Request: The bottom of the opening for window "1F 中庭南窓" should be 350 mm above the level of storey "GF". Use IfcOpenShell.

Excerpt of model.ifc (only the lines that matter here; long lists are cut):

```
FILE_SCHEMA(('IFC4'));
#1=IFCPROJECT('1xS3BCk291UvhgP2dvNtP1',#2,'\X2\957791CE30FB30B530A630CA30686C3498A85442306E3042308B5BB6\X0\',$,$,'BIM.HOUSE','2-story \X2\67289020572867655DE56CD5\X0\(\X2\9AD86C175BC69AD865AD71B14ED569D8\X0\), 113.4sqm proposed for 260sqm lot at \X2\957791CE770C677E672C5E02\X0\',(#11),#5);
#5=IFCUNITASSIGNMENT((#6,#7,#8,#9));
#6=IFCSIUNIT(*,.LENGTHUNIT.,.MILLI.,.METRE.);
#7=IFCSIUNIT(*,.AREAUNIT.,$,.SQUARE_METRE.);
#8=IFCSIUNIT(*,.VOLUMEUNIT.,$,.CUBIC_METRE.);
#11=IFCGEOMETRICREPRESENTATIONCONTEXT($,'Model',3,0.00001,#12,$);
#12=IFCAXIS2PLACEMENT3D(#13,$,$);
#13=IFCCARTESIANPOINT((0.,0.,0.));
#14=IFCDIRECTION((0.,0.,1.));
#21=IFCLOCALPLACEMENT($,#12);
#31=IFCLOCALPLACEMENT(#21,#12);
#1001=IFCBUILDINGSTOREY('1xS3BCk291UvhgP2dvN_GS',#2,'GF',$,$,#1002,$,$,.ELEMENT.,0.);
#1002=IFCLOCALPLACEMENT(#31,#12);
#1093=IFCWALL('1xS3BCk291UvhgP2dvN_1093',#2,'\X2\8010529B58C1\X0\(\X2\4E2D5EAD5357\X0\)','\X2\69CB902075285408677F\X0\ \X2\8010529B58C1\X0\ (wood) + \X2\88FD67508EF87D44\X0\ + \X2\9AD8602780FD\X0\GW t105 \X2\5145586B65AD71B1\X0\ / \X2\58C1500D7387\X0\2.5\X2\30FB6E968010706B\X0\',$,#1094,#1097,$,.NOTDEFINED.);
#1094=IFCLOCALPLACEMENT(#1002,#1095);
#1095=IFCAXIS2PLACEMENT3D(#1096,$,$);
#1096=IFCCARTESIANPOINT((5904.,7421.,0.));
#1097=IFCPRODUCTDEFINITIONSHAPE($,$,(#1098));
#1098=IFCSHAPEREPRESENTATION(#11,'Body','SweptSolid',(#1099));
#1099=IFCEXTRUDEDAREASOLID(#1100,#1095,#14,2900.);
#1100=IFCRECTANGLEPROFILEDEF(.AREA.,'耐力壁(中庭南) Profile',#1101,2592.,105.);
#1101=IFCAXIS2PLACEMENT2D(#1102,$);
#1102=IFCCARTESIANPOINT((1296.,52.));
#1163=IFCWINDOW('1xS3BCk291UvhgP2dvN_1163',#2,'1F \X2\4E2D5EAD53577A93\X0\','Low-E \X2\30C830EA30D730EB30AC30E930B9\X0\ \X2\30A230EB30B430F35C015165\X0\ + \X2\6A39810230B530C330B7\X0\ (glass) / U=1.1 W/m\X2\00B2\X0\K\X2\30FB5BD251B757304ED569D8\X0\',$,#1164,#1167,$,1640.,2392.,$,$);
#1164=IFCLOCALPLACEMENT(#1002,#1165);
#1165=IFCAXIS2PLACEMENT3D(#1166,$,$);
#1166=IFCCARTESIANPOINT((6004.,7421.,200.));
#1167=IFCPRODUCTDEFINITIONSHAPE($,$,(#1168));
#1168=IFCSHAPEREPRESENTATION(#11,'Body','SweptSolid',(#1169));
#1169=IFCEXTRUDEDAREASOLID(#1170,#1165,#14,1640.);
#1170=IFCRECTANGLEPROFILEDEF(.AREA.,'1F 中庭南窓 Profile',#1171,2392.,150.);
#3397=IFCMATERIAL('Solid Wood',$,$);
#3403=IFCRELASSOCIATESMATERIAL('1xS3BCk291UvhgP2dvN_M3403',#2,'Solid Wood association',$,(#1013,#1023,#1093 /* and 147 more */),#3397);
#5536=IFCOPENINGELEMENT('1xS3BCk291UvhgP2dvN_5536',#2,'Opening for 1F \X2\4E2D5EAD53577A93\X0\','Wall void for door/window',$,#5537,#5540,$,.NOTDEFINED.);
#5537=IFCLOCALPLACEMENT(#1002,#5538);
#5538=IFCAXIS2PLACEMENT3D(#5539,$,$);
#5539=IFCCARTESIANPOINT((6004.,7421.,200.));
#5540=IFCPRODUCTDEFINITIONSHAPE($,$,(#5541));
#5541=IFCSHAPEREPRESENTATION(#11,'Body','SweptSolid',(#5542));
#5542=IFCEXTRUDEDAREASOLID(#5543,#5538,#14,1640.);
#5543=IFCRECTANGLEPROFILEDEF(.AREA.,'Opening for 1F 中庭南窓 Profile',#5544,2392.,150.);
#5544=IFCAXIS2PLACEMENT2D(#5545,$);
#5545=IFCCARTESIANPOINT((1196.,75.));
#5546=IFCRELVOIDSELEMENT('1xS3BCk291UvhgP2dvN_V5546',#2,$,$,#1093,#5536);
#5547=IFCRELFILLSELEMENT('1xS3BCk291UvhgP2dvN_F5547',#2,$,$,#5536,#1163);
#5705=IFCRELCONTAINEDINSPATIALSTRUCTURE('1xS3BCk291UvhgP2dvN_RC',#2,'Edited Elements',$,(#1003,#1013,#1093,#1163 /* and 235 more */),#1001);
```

```python
import numpy as np
import ifcopenshell
import ifcopenshell.api.geometry
import ifcopenshell.geom
import ifcopenshell.util.element
import ifcopenshell.util.placement
import ifcopenshell.util.shape
import ifcopenshell.util.unit

model = ifcopenshell.open("model.ifc")
unit_scale = ifcopenshell.util.unit.calculate_unit_scale(model)

window = model.by_id(1163)
opening = window.FillsVoids[0].RelatingOpeningElement
storey = ifcopenshell.util.element.get_container(window, ifc_class="IfcBuildingStorey")
level = ifcopenshell.util.placement.get_local_placement(storey.ObjectPlacement)[2, 3]

# The opening's origin need not be at the sill, so measure its lowest point.
shape = ifcopenshell.geom.create_shape(ifcopenshell.geom.settings(), opening)
bottom = ifcopenshell.util.shape.get_shape_bottom_elevation(shape, shape.geometry) / unit_scale
dz = level + 0.35 / unit_scale - bottom

shift = np.array([0.0, 0.0, dz])
# The window is not placed relative to its opening, so move both.
for product in (opening, window):
    matrix = ifcopenshell.util.placement.get_local_placement(product.ObjectPlacement)
    matrix[:3, 3] += shift
    ifcopenshell.api.geometry.edit_object_placement(model, product=product, matrix=matrix, is_si=False)

print(f"moved by {dz * unit_scale:+.3f} m")

model.write("model-out.ifc")
```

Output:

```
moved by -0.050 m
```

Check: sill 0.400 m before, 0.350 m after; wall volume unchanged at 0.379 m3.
